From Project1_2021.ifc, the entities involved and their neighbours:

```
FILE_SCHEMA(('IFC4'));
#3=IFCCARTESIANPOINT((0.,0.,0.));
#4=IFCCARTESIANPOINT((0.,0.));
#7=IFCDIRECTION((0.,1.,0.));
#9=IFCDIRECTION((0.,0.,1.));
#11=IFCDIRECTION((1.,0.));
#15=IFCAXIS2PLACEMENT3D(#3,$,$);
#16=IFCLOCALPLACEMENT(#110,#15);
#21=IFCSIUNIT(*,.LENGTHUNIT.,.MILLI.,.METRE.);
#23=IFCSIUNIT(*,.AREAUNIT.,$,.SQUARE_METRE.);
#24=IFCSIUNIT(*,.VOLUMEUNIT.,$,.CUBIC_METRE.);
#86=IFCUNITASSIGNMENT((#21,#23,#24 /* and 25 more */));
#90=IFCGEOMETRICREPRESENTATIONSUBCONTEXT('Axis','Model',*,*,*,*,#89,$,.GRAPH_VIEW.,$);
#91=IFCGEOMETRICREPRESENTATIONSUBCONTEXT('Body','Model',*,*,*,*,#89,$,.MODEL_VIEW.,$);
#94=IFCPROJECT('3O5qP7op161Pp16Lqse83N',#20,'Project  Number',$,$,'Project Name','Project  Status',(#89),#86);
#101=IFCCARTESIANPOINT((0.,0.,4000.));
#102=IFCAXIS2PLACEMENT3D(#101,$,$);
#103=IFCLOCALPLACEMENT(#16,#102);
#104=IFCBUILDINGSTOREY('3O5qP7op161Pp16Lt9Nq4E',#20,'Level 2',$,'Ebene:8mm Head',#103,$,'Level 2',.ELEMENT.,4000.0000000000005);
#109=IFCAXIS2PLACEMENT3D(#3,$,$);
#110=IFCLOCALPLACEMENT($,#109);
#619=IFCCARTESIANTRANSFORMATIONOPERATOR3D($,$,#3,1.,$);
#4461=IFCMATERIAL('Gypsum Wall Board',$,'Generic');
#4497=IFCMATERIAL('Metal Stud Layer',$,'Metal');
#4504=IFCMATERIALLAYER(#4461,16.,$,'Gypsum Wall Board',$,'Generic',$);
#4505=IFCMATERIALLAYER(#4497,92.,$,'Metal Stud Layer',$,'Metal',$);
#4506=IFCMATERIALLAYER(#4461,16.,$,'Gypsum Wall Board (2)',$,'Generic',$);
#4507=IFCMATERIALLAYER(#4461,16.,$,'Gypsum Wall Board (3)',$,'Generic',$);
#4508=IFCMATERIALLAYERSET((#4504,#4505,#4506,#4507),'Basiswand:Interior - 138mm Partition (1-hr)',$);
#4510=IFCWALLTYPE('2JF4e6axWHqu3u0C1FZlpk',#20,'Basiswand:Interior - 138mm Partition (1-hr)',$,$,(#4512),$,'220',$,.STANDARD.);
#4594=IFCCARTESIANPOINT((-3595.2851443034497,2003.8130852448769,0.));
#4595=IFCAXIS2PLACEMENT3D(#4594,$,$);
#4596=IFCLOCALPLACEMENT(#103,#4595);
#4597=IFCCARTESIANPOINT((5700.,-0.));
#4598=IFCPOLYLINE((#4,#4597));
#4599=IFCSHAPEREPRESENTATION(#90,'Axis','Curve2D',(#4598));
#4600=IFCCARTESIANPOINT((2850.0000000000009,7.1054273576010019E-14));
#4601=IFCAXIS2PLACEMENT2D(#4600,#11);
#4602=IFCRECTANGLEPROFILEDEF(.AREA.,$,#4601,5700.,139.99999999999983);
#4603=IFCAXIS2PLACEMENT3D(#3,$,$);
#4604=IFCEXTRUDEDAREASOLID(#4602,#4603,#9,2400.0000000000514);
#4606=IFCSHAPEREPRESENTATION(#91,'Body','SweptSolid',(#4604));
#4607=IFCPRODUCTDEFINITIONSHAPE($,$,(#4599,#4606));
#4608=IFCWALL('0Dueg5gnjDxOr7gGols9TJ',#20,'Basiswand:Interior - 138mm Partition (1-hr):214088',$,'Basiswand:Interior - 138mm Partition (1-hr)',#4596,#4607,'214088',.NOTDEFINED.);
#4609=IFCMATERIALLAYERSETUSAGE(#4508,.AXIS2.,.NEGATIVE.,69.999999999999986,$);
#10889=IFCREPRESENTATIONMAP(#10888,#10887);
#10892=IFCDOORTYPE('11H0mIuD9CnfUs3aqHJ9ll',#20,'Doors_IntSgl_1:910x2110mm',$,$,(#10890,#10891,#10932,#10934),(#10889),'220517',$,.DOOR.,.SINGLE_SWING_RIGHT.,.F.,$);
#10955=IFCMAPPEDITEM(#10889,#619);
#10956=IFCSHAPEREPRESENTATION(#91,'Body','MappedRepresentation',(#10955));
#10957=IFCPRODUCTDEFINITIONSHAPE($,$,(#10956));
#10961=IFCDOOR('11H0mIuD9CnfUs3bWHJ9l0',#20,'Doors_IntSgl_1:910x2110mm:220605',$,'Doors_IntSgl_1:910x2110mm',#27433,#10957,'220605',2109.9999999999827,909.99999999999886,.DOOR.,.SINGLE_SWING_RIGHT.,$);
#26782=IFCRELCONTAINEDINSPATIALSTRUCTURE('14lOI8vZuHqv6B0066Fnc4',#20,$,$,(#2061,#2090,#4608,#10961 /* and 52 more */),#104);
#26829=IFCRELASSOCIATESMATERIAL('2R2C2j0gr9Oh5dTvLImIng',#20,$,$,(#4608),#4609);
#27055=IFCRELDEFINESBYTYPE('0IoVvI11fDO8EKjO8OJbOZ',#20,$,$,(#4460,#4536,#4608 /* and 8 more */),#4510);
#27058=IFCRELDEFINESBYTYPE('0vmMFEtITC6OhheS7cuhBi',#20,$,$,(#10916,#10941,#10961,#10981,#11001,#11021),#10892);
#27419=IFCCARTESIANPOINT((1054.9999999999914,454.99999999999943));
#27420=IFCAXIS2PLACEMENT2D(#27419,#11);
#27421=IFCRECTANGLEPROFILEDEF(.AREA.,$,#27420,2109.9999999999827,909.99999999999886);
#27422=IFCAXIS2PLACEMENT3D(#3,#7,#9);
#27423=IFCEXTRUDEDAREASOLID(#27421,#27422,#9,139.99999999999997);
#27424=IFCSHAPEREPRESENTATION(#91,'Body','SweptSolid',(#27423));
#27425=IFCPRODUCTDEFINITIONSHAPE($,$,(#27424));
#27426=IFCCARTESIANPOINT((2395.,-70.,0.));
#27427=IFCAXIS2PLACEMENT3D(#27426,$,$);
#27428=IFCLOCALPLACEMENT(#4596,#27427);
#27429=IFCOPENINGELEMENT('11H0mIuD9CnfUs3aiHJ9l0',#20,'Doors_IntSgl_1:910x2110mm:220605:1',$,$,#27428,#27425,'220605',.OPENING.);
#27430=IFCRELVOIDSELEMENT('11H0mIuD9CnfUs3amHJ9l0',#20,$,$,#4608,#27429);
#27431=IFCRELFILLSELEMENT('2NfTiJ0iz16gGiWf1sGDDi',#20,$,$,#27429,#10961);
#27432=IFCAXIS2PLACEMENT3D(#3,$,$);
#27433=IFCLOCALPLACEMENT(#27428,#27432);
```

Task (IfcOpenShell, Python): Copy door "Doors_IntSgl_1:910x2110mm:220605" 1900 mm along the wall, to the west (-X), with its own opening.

```python
import ifcopenshell
import ifcopenshell.api.feature
import ifcopenshell.api.geometry
import ifcopenshell.api.root
import ifcopenshell.geom
import ifcopenshell.util.element
import ifcopenshell.util.placement
import ifcopenshell.util.shape
import ifcopenshell.util.unit

model = ifcopenshell.open("Project1_2021.ifc")
unit_scale = ifcopenshell.util.unit.calculate_unit_scale(model)
settings = ifcopenshell.geom.settings()


def volume(element):
    """Net volume in cubic metres, openings subtracted."""
    shape = ifcopenshell.geom.create_shape(settings, element)
    return ifcopenshell.util.shape.get_volume(shape.geometry)


def reuse_history(source, copy):
    """copy_class also copies each property set's owner history, people and application; keep the originals."""
    for rel in copy.IsDefinedBy:
        if rel.is_a("IfcRelDefinesByProperties") and (history := rel.RelatingPropertyDefinition.OwnerHistory):
            rel.RelatingPropertyDefinition.OwnerHistory = source.OwnerHistory
            ifcopenshell.util.element.remove_deep2(model, history)


door = model.by_guid("11H0mIuD9CnfUs3bWHJ9l0")
opening = door.FillsVoids[0].RelatingOpeningElement
wall = opening.VoidsElements[0].RelatingBuildingElement
before = volume(wall)
shift = ifcopenshell.util.placement.get_local_placement(wall.ObjectPlacement)[:3, 0] * -1.9 / unit_scale

# copy_class copies the void relationship, type, container and properties, but no geometry.
new_opening = ifcopenshell.api.root.copy_class(model, product=opening)
new_opening.Representation = ifcopenshell.util.element.copy_deep(
    model, opening.Representation, exclude=["IfcGeometricRepresentationContext", "IfcRepresentationMap"]
)
new_opening.Name = "Doors_IntSgl_1:910x2110mm"
new_opening.Tag = None
new_door = ifcopenshell.api.root.copy_class(model, product=door)
new_door.Representation = ifcopenshell.util.element.copy_deep(
    model, door.Representation, exclude=["IfcGeometricRepresentationContext", "IfcRepresentationMap"]
)
new_door.Name = "Doors_IntSgl_1:910x2110mm"
new_door.Tag = None
reuse_history(door, new_door)
ifcopenshell.api.feature.add_filling(model, opening=new_opening, element=new_door)

for old, new in ((opening, new_opening), (door, new_door)):
    matrix = ifcopenshell.util.placement.get_local_placement(old.ObjectPlacement)
    matrix[:3, 3] += shift
    ifcopenshell.api.geometry.edit_object_placement(model, product=new, matrix=matrix, is_si=False)

after = volume(wall)

print(f"wall volume {before:.3f} -> {after:.3f} m3")

model.write("Project1_2021_updated.ifc")
```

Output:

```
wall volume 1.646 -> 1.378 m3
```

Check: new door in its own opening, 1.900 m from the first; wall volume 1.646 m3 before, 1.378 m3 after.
